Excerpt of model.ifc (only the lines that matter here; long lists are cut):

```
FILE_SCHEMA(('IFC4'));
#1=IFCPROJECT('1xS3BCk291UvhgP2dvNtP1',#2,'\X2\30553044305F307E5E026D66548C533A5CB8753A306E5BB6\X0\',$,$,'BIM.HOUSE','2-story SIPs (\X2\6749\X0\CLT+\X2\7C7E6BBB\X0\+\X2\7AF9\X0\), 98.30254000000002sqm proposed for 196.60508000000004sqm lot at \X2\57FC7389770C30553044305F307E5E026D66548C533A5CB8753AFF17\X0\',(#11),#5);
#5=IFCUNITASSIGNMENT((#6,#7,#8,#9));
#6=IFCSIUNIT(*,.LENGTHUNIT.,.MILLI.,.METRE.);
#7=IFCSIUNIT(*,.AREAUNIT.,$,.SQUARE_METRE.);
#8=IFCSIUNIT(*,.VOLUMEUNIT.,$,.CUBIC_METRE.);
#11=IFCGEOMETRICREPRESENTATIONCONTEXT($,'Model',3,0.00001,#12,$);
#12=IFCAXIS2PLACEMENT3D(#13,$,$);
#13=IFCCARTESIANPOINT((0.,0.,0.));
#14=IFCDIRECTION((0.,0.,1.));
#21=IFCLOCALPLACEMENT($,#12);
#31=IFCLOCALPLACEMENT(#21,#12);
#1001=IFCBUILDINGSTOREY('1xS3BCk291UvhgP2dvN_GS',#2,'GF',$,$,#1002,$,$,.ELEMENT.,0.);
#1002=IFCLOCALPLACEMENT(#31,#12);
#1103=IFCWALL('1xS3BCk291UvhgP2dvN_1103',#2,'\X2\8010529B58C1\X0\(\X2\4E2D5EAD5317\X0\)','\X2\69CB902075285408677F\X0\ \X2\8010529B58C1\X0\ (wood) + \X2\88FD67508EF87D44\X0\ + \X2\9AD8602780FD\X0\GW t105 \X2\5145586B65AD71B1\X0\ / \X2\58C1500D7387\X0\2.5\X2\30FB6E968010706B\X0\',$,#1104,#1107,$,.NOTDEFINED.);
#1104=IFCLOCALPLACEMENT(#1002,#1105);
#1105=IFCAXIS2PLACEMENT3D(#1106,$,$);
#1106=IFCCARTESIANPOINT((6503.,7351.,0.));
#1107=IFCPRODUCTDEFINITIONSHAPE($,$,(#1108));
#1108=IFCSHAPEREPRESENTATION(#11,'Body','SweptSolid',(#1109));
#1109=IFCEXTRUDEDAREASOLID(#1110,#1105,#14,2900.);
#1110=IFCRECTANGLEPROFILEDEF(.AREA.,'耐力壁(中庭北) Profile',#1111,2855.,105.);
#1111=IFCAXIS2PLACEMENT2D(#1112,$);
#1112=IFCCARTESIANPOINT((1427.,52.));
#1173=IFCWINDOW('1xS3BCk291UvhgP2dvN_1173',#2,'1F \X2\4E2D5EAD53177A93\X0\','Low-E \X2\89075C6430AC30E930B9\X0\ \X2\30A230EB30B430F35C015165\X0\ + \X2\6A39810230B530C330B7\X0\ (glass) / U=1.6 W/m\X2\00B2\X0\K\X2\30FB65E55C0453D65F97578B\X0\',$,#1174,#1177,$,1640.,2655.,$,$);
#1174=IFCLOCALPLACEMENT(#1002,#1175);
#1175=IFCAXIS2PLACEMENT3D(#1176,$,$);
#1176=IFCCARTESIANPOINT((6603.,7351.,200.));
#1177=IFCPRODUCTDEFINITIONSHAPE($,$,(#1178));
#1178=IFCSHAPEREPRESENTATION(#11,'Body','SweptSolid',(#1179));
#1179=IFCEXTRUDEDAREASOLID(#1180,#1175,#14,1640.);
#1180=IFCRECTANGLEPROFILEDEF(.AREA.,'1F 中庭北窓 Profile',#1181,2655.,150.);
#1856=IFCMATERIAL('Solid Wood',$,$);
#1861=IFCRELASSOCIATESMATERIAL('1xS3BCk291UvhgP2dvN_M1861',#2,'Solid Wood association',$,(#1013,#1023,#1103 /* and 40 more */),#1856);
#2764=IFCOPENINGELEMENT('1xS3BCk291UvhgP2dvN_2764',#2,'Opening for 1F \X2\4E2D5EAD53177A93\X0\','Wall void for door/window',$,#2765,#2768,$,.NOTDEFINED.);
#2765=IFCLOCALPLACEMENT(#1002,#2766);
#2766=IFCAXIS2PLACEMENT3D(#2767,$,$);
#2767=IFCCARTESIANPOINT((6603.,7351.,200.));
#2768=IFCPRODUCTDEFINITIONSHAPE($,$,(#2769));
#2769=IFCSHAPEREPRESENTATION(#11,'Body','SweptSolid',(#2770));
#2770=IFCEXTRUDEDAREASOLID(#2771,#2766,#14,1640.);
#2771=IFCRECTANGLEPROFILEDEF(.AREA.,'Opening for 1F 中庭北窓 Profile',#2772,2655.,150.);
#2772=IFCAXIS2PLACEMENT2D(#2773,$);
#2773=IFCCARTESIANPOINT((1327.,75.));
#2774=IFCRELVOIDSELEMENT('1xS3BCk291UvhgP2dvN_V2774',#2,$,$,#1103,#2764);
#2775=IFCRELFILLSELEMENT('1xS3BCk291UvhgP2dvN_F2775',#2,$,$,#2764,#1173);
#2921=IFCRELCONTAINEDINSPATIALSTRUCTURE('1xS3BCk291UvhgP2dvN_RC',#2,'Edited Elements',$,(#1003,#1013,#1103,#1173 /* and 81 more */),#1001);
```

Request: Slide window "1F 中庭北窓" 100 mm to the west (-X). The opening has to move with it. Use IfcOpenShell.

```python
import ifcopenshell
import ifcopenshell.api.geometry
import ifcopenshell.util.placement

model = ifcopenshell.open("model.ifc")

window = model.by_id(1173)
opening = window.FillsVoids[0].RelatingOpeningElement
wall = opening.VoidsElements[0].RelatingBuildingElement

wall_matrix = ifcopenshell.util.placement.get_local_placement(wall.ObjectPlacement)
shift = wall_matrix[:3, 0] * -100.0
before = ifcopenshell.util.placement.get_local_placement(window.ObjectPlacement)[:3, 3].copy()

# The window is not placed relative to its opening, so move both.
for product in (opening, window):
    matrix = ifcopenshell.util.placement.get_local_placement(product.ObjectPlacement)
    matrix[:3, 3] += shift
    ifcopenshell.api.geometry.edit_object_placement(model, product=product, matrix=matrix, is_si=False)

after = ifcopenshell.util.placement.get_local_placement(window.ObjectPlacement)[:3, 3]
print("window moved by", (after - before).round(3) + 0.0)

model.write("model_edited.ifc")
```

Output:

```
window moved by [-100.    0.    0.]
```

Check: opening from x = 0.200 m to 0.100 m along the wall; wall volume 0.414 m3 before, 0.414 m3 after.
